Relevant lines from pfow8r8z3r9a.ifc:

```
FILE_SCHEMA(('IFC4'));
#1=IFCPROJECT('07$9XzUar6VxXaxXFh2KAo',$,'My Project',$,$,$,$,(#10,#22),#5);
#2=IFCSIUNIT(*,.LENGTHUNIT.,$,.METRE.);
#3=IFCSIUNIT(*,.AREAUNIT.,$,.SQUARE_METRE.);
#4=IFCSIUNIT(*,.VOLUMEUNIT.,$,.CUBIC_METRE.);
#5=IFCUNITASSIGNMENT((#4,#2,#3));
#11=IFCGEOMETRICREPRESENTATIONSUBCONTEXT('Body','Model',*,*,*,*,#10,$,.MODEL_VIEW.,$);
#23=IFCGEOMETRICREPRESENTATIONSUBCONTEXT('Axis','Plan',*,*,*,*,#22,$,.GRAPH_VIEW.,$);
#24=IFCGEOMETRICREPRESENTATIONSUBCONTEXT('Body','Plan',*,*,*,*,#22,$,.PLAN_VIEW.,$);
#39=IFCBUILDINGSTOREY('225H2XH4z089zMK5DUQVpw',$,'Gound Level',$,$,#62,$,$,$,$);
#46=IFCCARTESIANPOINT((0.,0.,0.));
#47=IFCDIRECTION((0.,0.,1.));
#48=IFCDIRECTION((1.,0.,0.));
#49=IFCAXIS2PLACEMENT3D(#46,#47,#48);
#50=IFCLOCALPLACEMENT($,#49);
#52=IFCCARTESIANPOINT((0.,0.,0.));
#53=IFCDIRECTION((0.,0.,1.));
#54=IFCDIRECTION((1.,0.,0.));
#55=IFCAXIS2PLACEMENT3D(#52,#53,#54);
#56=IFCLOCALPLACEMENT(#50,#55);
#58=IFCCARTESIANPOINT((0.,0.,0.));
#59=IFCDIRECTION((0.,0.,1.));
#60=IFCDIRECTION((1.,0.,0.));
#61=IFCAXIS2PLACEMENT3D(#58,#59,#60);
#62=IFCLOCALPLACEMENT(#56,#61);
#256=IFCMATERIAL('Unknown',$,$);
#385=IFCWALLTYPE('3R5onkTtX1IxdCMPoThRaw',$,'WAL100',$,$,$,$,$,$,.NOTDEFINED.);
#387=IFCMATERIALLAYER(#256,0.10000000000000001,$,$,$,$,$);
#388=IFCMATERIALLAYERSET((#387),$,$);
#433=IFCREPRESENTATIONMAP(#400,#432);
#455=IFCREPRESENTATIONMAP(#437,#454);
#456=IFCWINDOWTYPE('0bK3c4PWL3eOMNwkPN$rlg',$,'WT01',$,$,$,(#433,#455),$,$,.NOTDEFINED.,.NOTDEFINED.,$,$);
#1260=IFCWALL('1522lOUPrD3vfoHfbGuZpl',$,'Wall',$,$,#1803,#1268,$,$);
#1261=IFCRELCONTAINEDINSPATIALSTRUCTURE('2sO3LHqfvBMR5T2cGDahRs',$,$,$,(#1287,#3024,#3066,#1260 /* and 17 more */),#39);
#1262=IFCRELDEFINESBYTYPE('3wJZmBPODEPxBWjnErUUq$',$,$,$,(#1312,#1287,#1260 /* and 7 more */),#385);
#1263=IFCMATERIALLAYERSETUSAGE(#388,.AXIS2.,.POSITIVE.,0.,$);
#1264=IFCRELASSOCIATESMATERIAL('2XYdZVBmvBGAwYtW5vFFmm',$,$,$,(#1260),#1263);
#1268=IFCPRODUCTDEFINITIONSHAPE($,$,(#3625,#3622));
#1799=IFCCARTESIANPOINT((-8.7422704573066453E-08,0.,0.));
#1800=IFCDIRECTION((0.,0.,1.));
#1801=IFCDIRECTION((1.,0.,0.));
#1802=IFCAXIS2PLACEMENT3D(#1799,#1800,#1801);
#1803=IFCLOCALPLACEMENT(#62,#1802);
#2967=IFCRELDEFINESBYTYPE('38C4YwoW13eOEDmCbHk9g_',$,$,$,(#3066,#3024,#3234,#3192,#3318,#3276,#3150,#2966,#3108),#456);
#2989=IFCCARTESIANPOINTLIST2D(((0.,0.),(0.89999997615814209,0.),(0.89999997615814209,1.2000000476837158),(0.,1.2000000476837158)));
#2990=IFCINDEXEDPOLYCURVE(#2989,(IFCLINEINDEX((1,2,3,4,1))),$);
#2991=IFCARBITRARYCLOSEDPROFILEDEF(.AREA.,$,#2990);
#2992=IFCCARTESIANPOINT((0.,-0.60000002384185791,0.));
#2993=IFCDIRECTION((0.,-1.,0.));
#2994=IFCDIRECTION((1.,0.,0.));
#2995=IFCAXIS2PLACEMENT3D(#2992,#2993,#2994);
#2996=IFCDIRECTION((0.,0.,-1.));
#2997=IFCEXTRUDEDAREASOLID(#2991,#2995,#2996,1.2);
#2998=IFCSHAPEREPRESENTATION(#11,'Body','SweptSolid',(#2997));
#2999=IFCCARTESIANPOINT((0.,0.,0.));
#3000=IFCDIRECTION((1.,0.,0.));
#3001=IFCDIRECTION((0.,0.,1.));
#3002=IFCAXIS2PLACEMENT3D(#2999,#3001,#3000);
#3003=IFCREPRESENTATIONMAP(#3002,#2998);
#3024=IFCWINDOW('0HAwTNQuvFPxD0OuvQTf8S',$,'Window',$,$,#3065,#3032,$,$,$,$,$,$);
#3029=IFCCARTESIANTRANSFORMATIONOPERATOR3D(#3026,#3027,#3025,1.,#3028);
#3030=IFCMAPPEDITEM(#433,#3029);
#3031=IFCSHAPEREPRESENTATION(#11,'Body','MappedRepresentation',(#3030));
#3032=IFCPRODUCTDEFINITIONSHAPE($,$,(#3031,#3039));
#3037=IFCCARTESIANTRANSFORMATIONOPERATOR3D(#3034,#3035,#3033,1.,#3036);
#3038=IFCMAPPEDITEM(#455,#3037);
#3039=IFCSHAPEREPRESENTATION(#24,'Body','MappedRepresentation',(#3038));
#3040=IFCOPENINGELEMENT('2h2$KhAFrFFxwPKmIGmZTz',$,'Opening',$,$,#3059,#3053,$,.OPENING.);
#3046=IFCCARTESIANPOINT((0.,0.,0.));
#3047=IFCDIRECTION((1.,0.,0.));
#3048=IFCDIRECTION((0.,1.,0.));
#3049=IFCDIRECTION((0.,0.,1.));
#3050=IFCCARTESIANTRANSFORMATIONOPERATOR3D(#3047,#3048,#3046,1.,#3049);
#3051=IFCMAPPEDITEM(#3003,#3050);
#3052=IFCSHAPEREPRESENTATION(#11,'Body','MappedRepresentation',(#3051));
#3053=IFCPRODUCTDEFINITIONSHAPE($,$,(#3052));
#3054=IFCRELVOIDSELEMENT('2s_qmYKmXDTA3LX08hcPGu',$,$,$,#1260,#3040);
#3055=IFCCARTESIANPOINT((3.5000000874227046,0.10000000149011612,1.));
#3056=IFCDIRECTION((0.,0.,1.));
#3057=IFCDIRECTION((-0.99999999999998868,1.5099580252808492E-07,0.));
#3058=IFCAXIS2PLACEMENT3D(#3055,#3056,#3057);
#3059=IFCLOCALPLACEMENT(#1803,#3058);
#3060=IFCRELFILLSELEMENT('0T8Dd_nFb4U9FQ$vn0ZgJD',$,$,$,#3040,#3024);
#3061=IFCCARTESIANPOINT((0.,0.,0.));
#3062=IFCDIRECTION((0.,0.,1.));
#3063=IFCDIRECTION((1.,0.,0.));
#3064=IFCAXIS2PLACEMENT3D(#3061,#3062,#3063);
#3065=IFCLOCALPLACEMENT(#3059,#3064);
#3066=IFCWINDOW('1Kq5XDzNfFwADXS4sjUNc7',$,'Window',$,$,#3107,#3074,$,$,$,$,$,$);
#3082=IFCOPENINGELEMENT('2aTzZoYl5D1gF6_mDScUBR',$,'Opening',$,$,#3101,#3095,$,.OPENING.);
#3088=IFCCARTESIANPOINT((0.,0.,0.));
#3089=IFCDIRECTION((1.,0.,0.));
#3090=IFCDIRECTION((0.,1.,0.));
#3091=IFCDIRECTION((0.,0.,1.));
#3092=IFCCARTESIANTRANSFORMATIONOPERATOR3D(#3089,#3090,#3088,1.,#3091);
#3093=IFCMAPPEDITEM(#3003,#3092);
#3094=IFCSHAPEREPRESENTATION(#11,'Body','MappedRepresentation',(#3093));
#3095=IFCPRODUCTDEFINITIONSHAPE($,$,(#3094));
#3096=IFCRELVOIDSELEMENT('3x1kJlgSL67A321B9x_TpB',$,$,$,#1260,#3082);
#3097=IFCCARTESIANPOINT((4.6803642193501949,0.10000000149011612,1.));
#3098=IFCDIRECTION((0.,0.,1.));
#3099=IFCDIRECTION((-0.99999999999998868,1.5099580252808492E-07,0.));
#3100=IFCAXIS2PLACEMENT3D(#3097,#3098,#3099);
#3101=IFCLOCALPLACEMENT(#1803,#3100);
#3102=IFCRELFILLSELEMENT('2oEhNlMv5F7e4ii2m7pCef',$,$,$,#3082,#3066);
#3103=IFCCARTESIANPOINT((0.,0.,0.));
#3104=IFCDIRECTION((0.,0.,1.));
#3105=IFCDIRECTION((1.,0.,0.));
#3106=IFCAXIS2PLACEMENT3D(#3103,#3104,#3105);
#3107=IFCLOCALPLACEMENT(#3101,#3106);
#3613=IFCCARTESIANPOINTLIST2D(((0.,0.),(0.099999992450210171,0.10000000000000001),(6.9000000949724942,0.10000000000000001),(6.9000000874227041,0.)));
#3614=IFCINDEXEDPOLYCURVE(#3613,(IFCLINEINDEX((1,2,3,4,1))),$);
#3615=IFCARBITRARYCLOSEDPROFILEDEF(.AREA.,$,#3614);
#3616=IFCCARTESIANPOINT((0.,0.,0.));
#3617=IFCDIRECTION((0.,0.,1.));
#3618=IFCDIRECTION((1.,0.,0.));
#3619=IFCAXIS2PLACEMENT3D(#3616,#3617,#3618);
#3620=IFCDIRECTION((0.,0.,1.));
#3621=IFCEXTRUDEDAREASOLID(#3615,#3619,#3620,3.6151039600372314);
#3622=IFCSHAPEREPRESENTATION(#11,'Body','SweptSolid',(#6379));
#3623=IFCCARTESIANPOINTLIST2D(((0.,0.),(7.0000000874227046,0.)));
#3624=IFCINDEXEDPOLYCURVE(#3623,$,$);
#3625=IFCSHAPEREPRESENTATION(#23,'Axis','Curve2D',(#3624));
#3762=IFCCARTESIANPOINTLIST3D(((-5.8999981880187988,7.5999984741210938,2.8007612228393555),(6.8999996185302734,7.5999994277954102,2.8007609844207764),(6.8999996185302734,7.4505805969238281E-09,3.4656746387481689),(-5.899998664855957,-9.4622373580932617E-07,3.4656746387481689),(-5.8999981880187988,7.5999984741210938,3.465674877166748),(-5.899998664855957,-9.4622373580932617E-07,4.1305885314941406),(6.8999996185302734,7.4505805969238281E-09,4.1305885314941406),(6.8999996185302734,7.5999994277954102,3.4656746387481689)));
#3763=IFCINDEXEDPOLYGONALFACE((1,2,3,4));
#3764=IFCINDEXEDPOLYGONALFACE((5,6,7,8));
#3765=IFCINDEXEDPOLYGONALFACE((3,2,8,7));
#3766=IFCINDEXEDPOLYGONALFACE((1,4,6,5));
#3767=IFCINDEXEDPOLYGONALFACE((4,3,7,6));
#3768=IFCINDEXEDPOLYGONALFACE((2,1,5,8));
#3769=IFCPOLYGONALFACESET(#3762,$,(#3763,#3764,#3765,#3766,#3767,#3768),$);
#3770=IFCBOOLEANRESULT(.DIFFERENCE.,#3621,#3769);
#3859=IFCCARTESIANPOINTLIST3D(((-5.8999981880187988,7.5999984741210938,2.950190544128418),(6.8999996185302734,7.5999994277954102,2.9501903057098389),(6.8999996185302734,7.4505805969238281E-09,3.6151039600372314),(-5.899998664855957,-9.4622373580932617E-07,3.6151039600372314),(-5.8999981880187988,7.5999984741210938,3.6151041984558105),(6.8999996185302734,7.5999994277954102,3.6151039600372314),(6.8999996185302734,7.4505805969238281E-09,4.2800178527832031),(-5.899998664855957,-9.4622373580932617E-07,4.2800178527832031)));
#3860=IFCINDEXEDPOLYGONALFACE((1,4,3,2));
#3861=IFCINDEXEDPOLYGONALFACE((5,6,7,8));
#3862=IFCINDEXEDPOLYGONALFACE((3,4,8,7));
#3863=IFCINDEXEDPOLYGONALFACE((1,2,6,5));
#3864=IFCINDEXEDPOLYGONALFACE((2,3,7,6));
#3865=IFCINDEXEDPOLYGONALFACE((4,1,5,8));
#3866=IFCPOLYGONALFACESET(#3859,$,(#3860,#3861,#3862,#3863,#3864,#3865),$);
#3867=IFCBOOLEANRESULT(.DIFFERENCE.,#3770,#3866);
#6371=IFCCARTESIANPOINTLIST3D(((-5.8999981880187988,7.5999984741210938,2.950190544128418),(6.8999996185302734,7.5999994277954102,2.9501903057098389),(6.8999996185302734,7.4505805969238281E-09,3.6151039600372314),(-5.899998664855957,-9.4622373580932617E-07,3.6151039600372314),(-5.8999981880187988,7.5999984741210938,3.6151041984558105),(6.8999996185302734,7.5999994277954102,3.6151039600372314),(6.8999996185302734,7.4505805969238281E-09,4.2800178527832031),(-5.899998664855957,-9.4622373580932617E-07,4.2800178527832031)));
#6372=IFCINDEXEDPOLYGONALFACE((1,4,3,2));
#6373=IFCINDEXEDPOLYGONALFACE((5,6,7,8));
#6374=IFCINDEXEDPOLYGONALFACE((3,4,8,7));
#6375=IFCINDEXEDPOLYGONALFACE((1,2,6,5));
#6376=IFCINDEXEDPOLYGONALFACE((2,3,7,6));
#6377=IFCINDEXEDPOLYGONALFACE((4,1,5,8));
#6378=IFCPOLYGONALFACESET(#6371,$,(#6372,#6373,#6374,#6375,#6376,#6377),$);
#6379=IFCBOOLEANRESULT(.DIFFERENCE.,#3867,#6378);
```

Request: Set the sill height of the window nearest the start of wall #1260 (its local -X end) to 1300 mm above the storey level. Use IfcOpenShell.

```python
import numpy as np
import ifcopenshell
import ifcopenshell.api.geometry
import ifcopenshell.geom
import ifcopenshell.util.element
import ifcopenshell.util.placement
import ifcopenshell.util.shape
import ifcopenshell.util.unit

model = ifcopenshell.open("pfow8r8z3r9a.ifc")
unit_scale = ifcopenshell.util.unit.calculate_unit_scale(model)

window = model.by_guid("0HAwTNQuvFPxD0OuvQTf8S")
opening = window.FillsVoids[0].RelatingOpeningElement
storey = ifcopenshell.util.element.get_container(window, ifc_class="IfcBuildingStorey")
level = ifcopenshell.util.placement.get_local_placement(storey.ObjectPlacement)[2, 3]

# The opening's origin need not be at the sill, so measure its lowest point.
shape = ifcopenshell.geom.create_shape(ifcopenshell.geom.settings(), opening)
bottom = ifcopenshell.util.shape.get_shape_bottom_elevation(shape, shape.geometry) / unit_scale
dz = level + 1.3 / unit_scale - bottom

shift = np.array([0.0, 0.0, dz])
# The window is placed relative to its opening, so it follows when the opening moves.
matrix = ifcopenshell.util.placement.get_local_placement(opening.ObjectPlacement)
matrix[:3, 3] += shift
ifcopenshell.api.geometry.edit_object_placement(
    model, product=opening, matrix=matrix, is_si=False, should_transform_children=True
)

print(f"moved by {dz * unit_scale:+.3f} m")

model.write("pfow8r8z3r9a_rev.ifc")
```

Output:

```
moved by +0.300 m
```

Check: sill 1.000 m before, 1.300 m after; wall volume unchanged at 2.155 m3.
